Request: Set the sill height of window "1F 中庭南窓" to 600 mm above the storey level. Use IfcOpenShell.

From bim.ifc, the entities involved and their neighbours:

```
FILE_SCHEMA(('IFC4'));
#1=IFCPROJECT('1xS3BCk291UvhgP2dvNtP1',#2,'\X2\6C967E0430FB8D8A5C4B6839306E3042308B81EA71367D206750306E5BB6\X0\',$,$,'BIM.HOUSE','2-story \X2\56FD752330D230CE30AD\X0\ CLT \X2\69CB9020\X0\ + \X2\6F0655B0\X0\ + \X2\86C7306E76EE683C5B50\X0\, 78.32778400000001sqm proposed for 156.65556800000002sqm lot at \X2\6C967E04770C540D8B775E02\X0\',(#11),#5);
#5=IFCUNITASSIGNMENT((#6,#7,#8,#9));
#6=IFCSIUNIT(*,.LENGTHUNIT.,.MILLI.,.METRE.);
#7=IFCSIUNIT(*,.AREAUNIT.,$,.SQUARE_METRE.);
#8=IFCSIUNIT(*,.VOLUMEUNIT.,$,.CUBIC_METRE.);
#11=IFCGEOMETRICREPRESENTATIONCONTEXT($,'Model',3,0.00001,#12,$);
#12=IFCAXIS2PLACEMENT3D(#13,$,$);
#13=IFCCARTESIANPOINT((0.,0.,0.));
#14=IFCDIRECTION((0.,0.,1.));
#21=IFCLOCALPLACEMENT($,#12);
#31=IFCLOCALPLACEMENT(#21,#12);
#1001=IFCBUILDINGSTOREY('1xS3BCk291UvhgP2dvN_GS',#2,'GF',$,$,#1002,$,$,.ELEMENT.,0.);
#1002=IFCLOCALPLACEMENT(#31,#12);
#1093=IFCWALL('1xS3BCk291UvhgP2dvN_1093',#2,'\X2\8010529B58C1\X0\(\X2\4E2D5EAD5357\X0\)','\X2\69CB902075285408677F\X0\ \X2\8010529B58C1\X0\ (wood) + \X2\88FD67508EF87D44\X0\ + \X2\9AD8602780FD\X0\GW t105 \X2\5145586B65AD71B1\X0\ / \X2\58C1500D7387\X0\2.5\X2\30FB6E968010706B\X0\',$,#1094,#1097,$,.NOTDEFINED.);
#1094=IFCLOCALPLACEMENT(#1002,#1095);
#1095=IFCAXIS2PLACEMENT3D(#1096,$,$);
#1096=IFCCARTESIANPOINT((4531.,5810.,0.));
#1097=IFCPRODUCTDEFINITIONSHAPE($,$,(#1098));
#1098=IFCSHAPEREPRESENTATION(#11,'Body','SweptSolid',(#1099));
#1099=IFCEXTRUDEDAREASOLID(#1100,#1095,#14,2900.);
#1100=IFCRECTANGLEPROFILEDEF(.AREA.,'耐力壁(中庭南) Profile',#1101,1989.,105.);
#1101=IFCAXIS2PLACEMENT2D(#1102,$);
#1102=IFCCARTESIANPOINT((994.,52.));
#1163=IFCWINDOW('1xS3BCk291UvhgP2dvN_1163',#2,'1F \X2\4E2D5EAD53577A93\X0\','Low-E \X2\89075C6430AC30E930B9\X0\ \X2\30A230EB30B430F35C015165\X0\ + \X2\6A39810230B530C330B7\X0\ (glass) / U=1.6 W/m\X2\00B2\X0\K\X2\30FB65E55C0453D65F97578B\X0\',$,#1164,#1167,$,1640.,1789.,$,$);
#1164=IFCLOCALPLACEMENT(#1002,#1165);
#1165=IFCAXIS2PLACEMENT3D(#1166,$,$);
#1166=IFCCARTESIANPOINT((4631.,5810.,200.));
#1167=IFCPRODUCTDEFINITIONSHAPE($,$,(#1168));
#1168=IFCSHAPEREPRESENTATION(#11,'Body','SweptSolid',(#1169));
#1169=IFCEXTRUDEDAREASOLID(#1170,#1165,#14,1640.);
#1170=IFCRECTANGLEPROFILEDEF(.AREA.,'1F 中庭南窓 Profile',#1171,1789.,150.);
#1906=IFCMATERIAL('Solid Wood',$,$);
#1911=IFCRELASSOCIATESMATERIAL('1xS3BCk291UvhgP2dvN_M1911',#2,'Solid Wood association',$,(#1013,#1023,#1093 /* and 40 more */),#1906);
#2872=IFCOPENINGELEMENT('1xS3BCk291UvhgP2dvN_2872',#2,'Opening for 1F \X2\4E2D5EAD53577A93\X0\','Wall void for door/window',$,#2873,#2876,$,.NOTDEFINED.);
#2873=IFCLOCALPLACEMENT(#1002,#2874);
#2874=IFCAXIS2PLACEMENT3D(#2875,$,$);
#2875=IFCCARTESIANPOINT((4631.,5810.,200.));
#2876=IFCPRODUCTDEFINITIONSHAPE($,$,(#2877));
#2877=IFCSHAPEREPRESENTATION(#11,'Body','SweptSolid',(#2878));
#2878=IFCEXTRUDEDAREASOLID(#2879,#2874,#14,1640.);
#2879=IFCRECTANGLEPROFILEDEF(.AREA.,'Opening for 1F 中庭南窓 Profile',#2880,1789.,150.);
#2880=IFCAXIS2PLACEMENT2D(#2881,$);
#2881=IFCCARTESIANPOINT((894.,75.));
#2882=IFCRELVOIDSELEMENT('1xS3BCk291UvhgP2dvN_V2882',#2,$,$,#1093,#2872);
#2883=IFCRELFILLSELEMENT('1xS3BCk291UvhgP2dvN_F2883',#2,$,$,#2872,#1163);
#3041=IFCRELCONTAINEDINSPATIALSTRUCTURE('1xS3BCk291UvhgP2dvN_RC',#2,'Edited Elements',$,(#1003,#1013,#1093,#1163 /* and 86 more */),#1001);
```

```python
import numpy as np
import ifcopenshell
import ifcopenshell.api.geometry
import ifcopenshell.geom
import ifcopenshell.util.element
import ifcopenshell.util.placement
import ifcopenshell.util.shape
import ifcopenshell.util.unit

model = ifcopenshell.open("bim.ifc")
unit_scale = ifcopenshell.util.unit.calculate_unit_scale(model)

window = model.by_id(1163)
opening = window.FillsVoids[0].RelatingOpeningElement
storey = ifcopenshell.util.element.get_container(window, ifc_class="IfcBuildingStorey")
level = ifcopenshell.util.placement.get_local_placement(storey.ObjectPlacement)[2, 3]

# The opening's origin need not be at the sill, so measure its lowest point.
shape = ifcopenshell.geom.create_shape(ifcopenshell.geom.settings(), opening)
bottom = ifcopenshell.util.shape.get_shape_bottom_elevation(shape, shape.geometry) / unit_scale
dz = level + 0.6 / unit_scale - bottom

shift = np.array([0.0, 0.0, dz])
# The window is not placed relative to its opening, so move both.
for product in (opening, window):
    matrix = ifcopenshell.util.placement.get_local_placement(product.ObjectPlacement)
    matrix[:3, 3] += shift
    ifcopenshell.api.geometry.edit_object_placement(model, product=product, matrix=matrix, is_si=False)

print(f"moved by {dz * unit_scale:+.3f} m")

model.write("bim_rev.ifc")
```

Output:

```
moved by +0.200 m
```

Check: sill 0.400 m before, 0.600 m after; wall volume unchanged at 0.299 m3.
